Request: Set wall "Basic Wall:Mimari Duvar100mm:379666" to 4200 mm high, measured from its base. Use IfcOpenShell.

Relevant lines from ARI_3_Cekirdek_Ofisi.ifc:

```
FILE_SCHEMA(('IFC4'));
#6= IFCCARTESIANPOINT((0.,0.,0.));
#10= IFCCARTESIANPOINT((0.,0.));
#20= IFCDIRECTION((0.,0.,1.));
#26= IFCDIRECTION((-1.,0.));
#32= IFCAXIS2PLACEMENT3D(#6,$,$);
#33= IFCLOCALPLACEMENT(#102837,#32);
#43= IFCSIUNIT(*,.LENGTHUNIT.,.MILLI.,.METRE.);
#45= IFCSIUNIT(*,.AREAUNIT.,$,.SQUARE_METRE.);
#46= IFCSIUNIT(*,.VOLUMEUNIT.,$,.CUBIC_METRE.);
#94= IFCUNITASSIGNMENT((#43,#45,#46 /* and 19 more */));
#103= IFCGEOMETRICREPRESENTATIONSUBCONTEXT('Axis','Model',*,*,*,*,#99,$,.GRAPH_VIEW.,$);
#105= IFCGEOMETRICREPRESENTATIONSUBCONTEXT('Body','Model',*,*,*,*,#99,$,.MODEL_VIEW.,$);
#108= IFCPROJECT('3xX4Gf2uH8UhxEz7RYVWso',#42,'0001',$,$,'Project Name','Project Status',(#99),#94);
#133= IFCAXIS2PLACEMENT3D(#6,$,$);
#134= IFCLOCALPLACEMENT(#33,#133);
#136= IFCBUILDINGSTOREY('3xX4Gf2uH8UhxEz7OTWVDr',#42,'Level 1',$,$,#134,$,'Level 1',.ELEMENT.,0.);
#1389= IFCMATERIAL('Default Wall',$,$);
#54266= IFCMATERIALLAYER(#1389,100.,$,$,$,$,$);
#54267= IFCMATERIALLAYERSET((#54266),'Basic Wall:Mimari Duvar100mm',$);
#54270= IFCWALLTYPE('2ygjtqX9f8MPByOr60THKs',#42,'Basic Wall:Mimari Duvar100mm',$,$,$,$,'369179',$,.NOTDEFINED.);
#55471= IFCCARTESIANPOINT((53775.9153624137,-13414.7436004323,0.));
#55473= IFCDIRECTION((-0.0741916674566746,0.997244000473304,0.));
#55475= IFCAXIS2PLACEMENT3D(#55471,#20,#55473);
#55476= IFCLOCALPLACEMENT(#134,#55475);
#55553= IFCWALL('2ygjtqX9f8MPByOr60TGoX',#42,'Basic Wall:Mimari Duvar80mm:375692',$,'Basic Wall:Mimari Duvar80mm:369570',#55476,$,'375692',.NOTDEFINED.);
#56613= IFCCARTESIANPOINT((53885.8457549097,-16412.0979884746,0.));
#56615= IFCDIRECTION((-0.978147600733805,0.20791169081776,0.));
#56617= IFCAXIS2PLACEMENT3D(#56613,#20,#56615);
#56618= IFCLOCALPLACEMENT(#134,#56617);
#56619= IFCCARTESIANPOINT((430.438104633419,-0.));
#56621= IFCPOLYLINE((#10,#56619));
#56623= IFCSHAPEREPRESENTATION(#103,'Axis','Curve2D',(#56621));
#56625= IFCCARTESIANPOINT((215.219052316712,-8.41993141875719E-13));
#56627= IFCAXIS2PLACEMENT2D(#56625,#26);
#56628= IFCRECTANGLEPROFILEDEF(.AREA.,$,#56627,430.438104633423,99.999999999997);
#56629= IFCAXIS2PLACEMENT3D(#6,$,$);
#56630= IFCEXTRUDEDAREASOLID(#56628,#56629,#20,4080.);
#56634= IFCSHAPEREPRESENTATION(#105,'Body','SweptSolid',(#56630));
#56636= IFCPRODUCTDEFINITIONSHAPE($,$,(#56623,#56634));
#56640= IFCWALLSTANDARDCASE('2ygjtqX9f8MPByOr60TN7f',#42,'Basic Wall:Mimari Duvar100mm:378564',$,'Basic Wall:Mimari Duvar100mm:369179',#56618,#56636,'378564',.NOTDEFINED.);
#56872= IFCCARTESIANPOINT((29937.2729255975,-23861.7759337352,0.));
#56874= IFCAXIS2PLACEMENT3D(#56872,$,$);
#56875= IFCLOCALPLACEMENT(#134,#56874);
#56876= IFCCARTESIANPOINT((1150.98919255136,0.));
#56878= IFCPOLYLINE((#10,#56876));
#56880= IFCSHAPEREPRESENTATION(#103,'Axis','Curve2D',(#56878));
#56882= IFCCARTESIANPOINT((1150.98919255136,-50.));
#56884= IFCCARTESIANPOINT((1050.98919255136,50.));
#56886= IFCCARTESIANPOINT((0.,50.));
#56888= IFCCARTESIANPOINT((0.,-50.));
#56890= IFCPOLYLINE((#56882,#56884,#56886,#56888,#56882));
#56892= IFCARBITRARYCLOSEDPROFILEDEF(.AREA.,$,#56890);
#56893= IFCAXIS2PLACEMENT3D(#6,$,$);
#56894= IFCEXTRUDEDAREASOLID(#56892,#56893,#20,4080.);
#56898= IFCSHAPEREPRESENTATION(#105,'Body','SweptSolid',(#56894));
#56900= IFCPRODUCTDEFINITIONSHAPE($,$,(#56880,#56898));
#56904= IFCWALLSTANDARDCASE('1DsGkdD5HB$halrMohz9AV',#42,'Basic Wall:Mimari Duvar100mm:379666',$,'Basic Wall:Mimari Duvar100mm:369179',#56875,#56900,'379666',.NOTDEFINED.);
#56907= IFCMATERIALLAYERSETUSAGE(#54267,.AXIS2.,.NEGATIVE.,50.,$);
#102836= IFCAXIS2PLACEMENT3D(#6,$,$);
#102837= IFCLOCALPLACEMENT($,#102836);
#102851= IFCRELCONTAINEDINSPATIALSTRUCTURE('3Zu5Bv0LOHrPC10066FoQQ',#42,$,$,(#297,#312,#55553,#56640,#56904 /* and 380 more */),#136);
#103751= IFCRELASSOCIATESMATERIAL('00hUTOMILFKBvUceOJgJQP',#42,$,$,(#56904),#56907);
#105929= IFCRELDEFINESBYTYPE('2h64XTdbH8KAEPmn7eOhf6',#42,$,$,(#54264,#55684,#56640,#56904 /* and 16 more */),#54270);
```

```python
import ifcopenshell
import ifcopenshell.geom
import ifcopenshell.util.representation
import ifcopenshell.util.shape
import ifcopenshell.util.unit

model = ifcopenshell.open("ARI_3_Cekirdek_Ofisi.ifc")
unit_scale = ifcopenshell.util.unit.calculate_unit_scale(model)
settings = ifcopenshell.geom.settings()


def volume(element):
    """Net volume in cubic metres, openings subtracted."""
    shape = ifcopenshell.geom.create_shape(settings, element)
    return ifcopenshell.util.shape.get_volume(shape.geometry)


wall = model.by_guid("1DsGkdD5HB$halrMohz9AV")
before = volume(wall)

body = ifcopenshell.util.representation.get_representation(wall, "Model", "Body")
solid = body.Items[0]
old_height = solid.Depth
solid.Depth = 4.2 / unit_scale
after = volume(wall)

print(f"height {old_height:g} -> {solid.Depth:g}, volume {before:.3f} -> {after:.3f} m3")

model.write("ARI_3_Cekirdek_Ofisi-out.ifc")
```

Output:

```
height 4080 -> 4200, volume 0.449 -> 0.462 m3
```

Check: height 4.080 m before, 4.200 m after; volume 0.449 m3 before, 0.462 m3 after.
